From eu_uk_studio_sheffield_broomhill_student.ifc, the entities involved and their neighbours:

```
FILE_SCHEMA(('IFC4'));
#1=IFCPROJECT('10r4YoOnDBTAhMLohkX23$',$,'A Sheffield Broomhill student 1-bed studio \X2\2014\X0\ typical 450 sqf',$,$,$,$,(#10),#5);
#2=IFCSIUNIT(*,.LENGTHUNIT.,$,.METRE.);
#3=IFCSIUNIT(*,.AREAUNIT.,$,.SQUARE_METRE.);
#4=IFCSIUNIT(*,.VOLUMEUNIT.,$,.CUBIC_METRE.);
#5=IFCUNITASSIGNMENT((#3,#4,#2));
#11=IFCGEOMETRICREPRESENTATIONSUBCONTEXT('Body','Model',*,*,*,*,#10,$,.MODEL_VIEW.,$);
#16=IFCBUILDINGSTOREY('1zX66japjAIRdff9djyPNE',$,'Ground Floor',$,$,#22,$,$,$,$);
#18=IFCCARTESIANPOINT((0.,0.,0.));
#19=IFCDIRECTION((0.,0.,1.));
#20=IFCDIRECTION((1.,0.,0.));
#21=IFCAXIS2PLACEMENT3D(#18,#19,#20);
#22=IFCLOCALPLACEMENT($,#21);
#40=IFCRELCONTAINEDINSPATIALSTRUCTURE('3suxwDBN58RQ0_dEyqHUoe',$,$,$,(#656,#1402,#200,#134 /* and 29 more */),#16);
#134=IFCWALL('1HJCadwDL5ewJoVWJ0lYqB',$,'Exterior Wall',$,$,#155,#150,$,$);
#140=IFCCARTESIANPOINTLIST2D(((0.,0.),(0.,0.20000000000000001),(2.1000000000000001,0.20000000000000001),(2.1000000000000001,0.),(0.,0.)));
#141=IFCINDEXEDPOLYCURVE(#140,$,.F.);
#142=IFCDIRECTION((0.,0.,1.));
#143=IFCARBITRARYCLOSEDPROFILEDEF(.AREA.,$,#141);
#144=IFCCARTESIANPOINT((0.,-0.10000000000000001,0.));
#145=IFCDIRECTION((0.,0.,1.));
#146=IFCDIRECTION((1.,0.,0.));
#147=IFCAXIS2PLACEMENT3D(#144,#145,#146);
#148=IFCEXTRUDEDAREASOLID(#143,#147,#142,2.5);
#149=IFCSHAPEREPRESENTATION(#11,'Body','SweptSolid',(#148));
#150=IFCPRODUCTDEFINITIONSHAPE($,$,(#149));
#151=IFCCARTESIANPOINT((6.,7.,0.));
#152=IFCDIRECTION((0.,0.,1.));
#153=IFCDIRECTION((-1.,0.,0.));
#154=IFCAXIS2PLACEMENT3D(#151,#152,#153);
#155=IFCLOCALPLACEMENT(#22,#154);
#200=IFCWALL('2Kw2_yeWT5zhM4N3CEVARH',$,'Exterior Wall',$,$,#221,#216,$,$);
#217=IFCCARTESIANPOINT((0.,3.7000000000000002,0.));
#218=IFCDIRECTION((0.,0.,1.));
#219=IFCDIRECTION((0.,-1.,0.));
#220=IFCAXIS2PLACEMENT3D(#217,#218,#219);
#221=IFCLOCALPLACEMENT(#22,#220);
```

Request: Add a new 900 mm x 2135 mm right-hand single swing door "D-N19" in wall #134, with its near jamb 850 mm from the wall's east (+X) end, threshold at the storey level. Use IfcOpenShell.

```python
import numpy as np
import ifcopenshell
import ifcopenshell.api.feature
import ifcopenshell.api.geometry
import ifcopenshell.api.root
import ifcopenshell.api.spatial
import ifcopenshell.geom
import ifcopenshell.util.element
import ifcopenshell.util.placement
import ifcopenshell.util.representation
import ifcopenshell.util.shape
import ifcopenshell.util.unit

model = ifcopenshell.open("eu_uk_studio_sheffield_broomhill_student.ifc")
unit_scale = ifcopenshell.util.unit.calculate_unit_scale(model)
settings = ifcopenshell.geom.settings()


def volume(element):
    """Net volume in cubic metres, openings subtracted."""
    shape = ifcopenshell.geom.create_shape(settings, element)
    return ifcopenshell.util.shape.get_volume(shape.geometry)


wall = model.by_guid("1HJCadwDL5ewJoVWJ0lYqB")
storey = ifcopenshell.util.element.get_container(wall, ifc_class="IfcBuildingStorey")
context = ifcopenshell.util.representation.get_context(model, "Model", "Body", "MODEL_VIEW")
before = volume(wall)

width, height, from_end, sill = 0.9, 2.135, 0.85, 0.0  # metres

# The wall runs along its own X axis, and the end named is its -X end.
wall_shape = ifcopenshell.geom.create_shape(settings, wall)
x, y, z = ifcopenshell.util.shape.get_vertices(wall_shape.geometry).T
start = x.min() + from_end
face, thickness = float(y.min()), float(y.max() - y.min())
wall_matrix = ifcopenshell.util.placement.get_local_placement(wall.ObjectPlacement)
level = ifcopenshell.util.placement.get_local_placement(storey.ObjectPlacement)[2, 3]


def in_wall(x, y):
    """Placement at x, y metres in the wall's axes, at sill height."""
    matrix = wall_matrix.copy()
    matrix[:, 3] = wall_matrix @ np.array([x / unit_scale, y / unit_scale, 0.0, 1.0])
    matrix[2, 3] = level + sill / unit_scale
    return matrix


# Opening: a box that overshoots both wall faces by 50 mm.
opening = ifcopenshell.api.root.create_entity(model, ifc_class="IfcOpeningElement", predefined_type="OPENING")
box = ifcopenshell.api.geometry.add_wall_representation(
    model, context=context, length=width, height=height, thickness=thickness + 0.1
)
ifcopenshell.api.geometry.assign_representation(model, product=opening, representation=box)
ifcopenshell.api.geometry.edit_object_placement(model, product=opening, matrix=in_wall(start, face - 0.05), is_si=False)
ifcopenshell.api.feature.add_feature(model, feature=opening, element=wall)

door = ifcopenshell.api.root.create_entity(model, ifc_class="IfcDoor", name="D-N19", predefined_type="DOOR")
door.OverallWidth, door.OverallHeight = width / unit_scale, height / unit_scale
door.OperationType = "SINGLE_SWING_RIGHT"
body = ifcopenshell.api.geometry.add_door_representation(
    model,
    context=context,
    overall_width=door.OverallWidth,
    overall_height=door.OverallHeight,
    operation_type="SINGLE_SWING_RIGHT",
    lining_properties={"LiningDepth": thickness / unit_scale, "ThresholdDepth": thickness / unit_scale},
)
ifcopenshell.api.geometry.assign_representation(model, product=door, representation=body)
ifcopenshell.api.spatial.assign_container(model, products=[door], relating_structure=storey)
ifcopenshell.api.feature.add_filling(model, opening=opening, element=door)

# The lining spans the wall, so the door starts at the wall face.
ifcopenshell.api.geometry.edit_object_placement(model, product=door, matrix=in_wall(start, face), is_si=False)

after = volume(wall)

print(f"wall volume {before:.3f} -> {after:.3f} m3")

model.write("eu_uk_studio_sheffield_broomhill_student-out.ifc")
```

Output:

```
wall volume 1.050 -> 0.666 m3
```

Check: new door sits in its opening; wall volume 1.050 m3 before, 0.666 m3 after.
